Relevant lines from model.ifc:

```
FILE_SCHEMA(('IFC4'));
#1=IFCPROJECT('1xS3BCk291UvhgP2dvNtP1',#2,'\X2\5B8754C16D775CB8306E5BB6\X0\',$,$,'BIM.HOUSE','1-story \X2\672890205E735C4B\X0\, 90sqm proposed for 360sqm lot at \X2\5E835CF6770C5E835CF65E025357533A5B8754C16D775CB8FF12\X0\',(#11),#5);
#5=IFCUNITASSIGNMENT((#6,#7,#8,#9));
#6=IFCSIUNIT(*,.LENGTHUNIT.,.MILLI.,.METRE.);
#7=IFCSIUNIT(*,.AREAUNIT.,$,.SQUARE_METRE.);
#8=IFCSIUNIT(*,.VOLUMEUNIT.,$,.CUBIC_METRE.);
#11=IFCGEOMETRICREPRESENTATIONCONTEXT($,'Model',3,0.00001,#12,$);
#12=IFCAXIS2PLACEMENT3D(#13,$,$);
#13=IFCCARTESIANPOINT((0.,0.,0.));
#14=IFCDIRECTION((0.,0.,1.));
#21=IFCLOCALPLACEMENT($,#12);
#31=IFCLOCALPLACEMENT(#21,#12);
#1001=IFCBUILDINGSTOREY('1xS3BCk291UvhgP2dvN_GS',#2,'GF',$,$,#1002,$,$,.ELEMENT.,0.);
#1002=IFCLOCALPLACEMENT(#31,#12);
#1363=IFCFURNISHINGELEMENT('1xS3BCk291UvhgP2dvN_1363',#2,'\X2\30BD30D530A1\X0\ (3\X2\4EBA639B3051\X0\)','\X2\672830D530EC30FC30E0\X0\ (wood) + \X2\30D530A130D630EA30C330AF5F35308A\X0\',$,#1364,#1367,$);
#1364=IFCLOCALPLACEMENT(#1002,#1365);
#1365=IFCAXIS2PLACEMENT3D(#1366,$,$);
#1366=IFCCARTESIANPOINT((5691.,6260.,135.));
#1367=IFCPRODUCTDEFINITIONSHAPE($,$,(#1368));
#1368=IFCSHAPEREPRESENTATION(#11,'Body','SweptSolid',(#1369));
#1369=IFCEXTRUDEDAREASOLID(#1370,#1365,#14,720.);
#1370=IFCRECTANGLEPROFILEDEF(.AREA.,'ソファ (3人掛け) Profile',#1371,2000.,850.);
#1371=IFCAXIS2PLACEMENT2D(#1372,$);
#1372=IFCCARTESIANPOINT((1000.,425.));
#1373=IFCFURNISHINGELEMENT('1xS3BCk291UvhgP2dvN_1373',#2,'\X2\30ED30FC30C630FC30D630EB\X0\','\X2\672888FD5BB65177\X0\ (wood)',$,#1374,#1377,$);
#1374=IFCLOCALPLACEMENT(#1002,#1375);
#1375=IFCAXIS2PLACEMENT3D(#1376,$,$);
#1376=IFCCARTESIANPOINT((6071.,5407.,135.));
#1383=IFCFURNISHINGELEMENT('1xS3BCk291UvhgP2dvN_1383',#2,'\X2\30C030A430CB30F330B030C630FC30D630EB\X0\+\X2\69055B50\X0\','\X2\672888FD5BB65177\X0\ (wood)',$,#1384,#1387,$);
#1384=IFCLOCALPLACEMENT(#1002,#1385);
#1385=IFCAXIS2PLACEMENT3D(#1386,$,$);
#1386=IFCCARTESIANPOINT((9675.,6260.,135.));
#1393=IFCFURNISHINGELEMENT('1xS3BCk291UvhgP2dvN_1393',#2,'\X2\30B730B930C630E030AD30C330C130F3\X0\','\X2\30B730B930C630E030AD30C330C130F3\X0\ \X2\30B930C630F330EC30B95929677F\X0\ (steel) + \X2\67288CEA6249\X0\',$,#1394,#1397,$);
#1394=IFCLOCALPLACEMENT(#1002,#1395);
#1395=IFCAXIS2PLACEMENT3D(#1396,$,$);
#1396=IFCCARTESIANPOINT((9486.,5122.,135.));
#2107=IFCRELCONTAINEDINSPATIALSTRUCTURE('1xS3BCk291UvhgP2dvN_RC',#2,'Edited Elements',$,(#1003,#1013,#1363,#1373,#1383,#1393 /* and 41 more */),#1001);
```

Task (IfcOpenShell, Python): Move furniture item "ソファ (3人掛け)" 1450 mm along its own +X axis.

```python
import ifcopenshell
import ifcopenshell.api.geometry
import ifcopenshell.util.placement
import ifcopenshell.util.unit

model = ifcopenshell.open("model.ifc")
unit_scale = ifcopenshell.util.unit.calculate_unit_scale(model)

item = model.by_guid("1xS3BCk291UvhgP2dvN_1363")
matrix = ifcopenshell.util.placement.get_local_placement(item.ObjectPlacement)
matrix[:3, 3] += matrix[:3, 0] * 1.45 / unit_scale
ifcopenshell.api.geometry.edit_object_placement(model, product=item, matrix=matrix, is_si=False)

print(ifcopenshell.util.placement.get_local_placement(item.ObjectPlacement).round(3) + 0.0)

model.write("model-out.ifc")
```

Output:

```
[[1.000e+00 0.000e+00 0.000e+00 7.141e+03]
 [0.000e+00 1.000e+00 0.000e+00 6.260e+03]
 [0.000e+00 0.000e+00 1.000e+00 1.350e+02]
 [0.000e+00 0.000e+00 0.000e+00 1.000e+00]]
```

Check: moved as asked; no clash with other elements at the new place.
